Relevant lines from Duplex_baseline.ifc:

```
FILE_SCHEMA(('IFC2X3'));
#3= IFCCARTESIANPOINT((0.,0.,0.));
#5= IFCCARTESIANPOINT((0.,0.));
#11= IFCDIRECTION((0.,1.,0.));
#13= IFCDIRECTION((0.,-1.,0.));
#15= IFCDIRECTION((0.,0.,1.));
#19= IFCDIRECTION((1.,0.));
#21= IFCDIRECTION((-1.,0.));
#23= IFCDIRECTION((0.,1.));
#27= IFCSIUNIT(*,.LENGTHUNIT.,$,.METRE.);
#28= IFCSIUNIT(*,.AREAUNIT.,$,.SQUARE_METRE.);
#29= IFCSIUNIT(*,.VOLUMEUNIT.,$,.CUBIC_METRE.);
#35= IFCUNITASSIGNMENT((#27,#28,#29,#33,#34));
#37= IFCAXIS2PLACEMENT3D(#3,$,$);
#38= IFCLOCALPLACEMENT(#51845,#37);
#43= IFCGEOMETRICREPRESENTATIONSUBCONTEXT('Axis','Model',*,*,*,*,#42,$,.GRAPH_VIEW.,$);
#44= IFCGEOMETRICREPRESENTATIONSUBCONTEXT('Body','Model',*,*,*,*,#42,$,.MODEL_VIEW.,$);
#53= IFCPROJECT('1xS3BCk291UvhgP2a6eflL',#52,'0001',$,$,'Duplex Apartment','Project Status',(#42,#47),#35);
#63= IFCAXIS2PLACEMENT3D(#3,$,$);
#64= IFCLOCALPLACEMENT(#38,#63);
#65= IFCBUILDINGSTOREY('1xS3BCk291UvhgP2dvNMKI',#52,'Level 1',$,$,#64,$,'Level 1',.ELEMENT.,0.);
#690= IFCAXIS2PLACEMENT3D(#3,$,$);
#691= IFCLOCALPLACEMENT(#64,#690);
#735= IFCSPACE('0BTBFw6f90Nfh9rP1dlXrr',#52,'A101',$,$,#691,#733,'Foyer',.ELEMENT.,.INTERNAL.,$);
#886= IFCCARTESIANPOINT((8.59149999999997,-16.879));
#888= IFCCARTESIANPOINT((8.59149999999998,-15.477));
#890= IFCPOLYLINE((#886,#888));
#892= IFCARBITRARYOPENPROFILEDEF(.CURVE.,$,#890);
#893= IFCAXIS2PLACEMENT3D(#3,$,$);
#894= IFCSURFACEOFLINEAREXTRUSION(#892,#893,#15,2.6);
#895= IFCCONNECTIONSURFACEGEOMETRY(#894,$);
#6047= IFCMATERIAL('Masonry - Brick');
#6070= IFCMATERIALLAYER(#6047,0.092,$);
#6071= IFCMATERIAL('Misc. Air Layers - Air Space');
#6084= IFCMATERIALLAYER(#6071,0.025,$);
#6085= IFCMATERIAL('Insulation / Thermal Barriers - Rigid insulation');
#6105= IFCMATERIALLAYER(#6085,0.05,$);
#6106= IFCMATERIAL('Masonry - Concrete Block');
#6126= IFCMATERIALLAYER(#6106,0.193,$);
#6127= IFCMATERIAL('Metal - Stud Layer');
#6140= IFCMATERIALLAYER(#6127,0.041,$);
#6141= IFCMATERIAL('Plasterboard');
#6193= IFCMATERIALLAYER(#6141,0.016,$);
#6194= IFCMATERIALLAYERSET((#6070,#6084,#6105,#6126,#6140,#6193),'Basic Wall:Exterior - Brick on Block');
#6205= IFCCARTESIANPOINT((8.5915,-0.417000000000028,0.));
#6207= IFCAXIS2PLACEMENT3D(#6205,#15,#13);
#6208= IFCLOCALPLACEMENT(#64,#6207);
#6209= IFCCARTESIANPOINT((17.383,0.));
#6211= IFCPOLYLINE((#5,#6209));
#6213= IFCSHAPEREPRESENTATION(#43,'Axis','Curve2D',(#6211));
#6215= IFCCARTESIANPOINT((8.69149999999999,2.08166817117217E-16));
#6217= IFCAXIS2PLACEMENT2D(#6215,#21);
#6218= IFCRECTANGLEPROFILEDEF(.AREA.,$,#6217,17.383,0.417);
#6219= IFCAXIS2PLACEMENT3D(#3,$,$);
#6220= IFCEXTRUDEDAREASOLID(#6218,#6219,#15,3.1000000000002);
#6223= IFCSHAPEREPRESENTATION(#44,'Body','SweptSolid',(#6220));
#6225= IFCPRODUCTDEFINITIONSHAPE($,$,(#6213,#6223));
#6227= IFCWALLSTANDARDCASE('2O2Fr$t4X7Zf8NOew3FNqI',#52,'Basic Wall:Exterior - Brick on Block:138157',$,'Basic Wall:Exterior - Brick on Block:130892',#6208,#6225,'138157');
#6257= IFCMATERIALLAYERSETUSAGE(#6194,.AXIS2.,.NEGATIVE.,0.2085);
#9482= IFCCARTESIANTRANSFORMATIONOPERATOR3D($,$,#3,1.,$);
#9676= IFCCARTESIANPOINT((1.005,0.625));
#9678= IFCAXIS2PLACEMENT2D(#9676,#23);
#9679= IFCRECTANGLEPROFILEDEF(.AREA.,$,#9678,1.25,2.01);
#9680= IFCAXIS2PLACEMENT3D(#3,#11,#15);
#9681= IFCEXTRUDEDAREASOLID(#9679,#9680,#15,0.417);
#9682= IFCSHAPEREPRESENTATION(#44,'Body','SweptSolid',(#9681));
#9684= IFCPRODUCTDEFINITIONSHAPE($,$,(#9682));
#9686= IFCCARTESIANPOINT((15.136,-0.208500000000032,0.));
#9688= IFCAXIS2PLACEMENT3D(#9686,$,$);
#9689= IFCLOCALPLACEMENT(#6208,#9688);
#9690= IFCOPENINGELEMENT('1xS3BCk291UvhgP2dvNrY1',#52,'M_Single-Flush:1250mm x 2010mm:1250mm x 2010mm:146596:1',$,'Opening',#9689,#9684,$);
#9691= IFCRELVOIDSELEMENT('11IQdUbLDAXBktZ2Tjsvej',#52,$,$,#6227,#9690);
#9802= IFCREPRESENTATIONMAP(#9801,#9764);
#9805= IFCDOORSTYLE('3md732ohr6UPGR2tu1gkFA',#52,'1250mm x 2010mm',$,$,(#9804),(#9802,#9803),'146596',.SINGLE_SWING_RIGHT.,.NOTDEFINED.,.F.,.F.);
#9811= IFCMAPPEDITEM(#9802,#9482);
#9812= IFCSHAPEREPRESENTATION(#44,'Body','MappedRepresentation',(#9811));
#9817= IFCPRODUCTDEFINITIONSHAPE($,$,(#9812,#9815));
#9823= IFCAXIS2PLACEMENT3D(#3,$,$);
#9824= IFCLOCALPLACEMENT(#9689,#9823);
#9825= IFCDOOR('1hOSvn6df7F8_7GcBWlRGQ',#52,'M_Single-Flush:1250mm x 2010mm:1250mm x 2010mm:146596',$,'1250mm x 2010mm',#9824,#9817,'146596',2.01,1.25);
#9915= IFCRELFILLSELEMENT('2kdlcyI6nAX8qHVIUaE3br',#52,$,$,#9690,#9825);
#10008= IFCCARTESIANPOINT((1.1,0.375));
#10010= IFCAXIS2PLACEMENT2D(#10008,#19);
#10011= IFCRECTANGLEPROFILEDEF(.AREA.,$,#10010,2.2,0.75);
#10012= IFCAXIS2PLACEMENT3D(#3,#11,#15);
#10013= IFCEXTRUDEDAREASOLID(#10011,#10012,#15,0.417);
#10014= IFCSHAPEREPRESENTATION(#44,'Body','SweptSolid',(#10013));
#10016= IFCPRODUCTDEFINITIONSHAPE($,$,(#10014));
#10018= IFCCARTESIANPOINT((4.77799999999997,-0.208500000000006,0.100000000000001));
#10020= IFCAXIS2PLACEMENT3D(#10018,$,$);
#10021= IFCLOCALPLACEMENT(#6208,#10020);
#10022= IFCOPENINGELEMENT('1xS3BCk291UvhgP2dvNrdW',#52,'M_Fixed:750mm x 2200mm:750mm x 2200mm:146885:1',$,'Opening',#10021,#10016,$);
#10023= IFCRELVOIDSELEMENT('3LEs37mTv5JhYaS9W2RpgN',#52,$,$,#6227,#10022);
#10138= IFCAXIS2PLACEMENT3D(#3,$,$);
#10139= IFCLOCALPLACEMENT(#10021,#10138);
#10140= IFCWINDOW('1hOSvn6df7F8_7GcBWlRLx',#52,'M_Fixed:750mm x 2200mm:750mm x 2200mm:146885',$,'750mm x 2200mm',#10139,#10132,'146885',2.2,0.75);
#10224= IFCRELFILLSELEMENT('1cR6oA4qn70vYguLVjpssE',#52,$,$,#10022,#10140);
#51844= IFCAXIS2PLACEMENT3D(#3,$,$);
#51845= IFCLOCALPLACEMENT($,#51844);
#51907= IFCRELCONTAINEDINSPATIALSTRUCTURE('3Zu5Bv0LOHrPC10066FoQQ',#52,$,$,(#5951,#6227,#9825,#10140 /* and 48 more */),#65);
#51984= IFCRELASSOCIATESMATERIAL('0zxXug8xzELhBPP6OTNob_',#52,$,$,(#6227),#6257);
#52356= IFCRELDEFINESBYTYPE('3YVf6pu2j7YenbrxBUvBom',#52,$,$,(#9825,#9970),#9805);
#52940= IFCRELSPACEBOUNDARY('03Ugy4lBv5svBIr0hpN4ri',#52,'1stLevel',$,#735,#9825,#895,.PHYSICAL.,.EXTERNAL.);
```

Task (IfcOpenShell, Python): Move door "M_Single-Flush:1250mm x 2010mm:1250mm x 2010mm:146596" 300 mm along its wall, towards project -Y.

```python
import numpy as np
import ifcopenshell
import ifcopenshell.api.geometry
import ifcopenshell.util.placement
import ifcopenshell.util.unit

model = ifcopenshell.open("Duplex_baseline.ifc")
unit_scale = ifcopenshell.util.unit.calculate_unit_scale(model)

door = model.by_guid("1hOSvn6df7F8_7GcBWlRGQ")
opening = door.FillsVoids[0].RelatingOpeningElement
wall = opening.VoidsElements[0].RelatingBuildingElement

wall_matrix = ifcopenshell.util.placement.get_local_placement(wall.ObjectPlacement)
shift = wall_matrix[:3, 0] * 0.3 / unit_scale
before = ifcopenshell.util.placement.get_local_placement(door.ObjectPlacement)[:3, 3].copy()

# The door is placed relative to its opening, so it follows when the opening moves.
matrix = ifcopenshell.util.placement.get_local_placement(opening.ObjectPlacement)
matrix[:3, 3] += shift
ifcopenshell.api.geometry.edit_object_placement(
    model, product=opening, matrix=matrix, is_si=False, should_transform_children=True
)

# Space boundary surfaces are stored in each space's coordinates; move them too.
for rel in door.ProvidesBoundaries:
    if not rel.ConnectionGeometry:
        continue
    surface = rel.ConnectionGeometry.SurfaceOnRelatingElement
    space_matrix = ifcopenshell.util.placement.get_local_placement(rel.RelatingSpace.ObjectPlacement)
    point = np.array(surface.Position.Location.Coordinates) + space_matrix[:3, :3].T @ shift
    surface.Position = model.createIfcAxis2Placement3D(
        model.createIfcCartesianPoint(point.tolist()), surface.Position.Axis, surface.Position.RefDirection
    )

after = ifcopenshell.util.placement.get_local_placement(door.ObjectPlacement)[:3, 3]
print("door moved by", (after - before).round(3) + 0.0)

model.write("Duplex_baseline-out.ifc")
```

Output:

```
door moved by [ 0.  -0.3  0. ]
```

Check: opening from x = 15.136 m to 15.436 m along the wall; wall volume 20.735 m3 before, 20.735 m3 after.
